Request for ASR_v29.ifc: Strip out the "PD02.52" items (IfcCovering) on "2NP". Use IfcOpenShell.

First a look at what the model holds.

```python
import ifcopenshell
import ifcopenshell.util.element

model = ifcopenshell.open("ASR_v29.ifc")
print(model.schema)
storey = next(s for s in model.by_type("IfcBuildingStorey") if s.Name == "2NP")
coverings = [e for e in ifcopenshell.util.element.get_decomposition(storey) if e.is_a("IfcCovering")]
seen = {}
for e in coverings:
    element_type = ifcopenshell.util.element.get_type(e)
    name = element_type.Name if element_type not in (None, e) else None
    seen[name] = seen.get(name, 0) + 1
for name, count in sorted(seen.items(), key=str):
    print(count, "x", name)
```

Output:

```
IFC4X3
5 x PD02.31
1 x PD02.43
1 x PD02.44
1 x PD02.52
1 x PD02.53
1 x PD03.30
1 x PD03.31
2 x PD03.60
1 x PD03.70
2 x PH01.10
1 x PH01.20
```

```python
import ifcopenshell
import ifcopenshell.api.root
import ifcopenshell.util.element

model = ifcopenshell.open("ASR_v29.ifc")

storey = next(s for s in model.by_type("IfcBuildingStorey") if s.Name == "2NP")
coverings = [e for e in ifcopenshell.util.element.get_decomposition(storey) if e.is_a("IfcCovering")]
targets = [e for e in coverings if (t := ifcopenshell.util.element.get_type(e)) not in (None, e) and t.Name == "PD02.52"]

for e in targets:
    ifcopenshell.api.root.remove_product(model, product=e)
print(len(targets), "removed")

model.write("ASR_v29-out.ifc")
```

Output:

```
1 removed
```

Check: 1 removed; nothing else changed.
